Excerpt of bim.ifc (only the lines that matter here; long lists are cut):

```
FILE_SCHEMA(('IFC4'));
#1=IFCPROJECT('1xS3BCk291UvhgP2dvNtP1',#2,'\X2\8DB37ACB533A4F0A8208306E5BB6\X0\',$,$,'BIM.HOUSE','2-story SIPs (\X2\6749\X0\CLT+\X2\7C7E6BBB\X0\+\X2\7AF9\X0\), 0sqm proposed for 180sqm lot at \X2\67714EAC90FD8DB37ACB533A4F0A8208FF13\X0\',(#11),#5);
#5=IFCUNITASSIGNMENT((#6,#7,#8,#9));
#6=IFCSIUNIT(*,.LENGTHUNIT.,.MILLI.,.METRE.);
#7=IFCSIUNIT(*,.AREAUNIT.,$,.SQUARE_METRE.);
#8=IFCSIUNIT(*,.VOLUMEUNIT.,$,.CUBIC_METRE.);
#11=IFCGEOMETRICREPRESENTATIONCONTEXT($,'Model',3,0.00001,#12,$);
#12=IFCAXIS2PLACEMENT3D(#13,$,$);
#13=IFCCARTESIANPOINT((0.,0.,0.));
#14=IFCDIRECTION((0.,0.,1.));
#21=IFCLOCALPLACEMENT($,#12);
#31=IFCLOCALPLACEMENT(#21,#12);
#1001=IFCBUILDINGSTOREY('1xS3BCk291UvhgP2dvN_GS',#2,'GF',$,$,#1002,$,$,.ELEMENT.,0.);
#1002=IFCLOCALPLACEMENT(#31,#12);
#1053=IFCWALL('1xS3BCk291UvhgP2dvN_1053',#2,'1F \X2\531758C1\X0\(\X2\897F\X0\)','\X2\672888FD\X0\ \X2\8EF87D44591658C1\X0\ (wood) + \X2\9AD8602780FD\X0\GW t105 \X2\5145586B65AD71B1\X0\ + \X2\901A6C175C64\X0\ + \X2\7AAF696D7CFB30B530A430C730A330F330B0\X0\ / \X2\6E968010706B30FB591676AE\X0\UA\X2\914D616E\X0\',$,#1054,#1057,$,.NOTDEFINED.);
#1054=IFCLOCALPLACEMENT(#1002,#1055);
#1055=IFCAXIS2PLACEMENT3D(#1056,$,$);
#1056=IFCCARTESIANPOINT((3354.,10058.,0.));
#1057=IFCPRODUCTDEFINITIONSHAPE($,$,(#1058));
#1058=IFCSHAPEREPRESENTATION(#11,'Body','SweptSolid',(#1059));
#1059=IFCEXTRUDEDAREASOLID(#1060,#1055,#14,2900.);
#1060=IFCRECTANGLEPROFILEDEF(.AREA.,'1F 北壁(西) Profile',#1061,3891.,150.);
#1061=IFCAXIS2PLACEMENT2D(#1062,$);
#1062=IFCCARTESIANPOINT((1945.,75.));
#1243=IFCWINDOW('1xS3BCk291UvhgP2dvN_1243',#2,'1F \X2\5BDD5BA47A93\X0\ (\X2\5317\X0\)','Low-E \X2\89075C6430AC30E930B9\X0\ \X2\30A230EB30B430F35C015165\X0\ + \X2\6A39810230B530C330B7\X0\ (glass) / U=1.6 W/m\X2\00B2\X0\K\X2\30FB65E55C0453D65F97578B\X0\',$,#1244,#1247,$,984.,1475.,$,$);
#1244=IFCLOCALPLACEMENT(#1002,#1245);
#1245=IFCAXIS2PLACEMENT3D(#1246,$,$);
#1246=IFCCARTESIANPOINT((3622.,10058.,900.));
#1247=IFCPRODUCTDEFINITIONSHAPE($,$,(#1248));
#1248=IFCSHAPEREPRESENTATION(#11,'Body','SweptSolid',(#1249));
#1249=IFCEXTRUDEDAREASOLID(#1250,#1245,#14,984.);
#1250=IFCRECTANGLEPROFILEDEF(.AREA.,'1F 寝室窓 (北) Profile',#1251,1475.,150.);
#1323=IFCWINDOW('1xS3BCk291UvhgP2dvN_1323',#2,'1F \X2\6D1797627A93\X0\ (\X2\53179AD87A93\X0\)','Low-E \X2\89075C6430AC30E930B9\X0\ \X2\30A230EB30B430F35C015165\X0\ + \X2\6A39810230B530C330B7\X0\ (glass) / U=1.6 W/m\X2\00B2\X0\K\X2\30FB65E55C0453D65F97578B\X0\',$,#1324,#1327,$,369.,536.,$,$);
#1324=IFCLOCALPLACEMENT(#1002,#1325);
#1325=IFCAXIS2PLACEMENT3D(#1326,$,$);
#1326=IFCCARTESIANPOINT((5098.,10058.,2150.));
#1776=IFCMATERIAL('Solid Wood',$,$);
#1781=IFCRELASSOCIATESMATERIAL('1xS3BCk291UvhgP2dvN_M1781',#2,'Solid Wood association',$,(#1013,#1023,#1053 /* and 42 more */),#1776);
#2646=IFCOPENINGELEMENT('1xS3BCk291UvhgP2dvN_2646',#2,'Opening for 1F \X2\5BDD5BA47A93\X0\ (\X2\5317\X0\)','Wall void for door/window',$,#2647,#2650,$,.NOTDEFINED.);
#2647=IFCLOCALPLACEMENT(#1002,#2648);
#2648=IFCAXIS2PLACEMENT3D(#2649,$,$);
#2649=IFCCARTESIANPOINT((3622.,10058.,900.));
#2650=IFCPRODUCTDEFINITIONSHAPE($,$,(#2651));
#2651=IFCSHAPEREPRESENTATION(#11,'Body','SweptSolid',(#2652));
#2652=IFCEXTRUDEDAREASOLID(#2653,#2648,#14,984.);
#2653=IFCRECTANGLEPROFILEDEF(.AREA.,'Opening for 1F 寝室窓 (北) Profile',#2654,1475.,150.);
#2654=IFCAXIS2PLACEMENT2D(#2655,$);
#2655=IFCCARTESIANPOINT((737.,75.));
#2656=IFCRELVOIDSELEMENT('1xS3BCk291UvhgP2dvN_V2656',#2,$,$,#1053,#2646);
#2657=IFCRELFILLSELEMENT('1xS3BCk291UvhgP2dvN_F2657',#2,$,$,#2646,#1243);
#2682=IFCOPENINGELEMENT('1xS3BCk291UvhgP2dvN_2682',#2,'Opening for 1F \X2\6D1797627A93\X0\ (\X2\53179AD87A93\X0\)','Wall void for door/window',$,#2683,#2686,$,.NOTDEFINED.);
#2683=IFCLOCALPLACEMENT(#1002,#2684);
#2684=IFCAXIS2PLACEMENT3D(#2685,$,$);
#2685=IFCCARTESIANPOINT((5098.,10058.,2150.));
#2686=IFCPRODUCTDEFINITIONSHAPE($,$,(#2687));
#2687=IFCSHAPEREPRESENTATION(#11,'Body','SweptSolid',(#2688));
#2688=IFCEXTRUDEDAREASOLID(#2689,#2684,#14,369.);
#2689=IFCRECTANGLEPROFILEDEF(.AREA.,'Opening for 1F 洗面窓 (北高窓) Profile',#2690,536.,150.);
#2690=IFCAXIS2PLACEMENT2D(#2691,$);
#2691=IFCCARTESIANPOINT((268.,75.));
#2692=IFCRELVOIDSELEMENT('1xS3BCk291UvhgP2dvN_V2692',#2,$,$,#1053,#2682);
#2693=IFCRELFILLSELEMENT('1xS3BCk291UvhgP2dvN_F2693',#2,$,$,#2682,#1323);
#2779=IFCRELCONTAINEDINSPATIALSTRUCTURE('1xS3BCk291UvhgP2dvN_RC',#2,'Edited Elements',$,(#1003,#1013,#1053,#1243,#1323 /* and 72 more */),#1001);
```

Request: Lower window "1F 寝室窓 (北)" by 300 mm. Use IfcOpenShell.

```python
import numpy as np
import ifcopenshell
import ifcopenshell.api.geometry
import ifcopenshell.util.placement
import ifcopenshell.util.unit

model = ifcopenshell.open("bim.ifc")
unit_scale = ifcopenshell.util.unit.calculate_unit_scale(model)

window = model.by_guid("1xS3BCk291UvhgP2dvN_1243")
opening = window.FillsVoids[0].RelatingOpeningElement
dz = -0.3 / unit_scale

shift = np.array([0.0, 0.0, dz])
# The window is not placed relative to its opening, so move both.
for product in (opening, window):
    matrix = ifcopenshell.util.placement.get_local_placement(product.ObjectPlacement)
    matrix[:3, 3] += shift
    ifcopenshell.api.geometry.edit_object_placement(model, product=product, matrix=matrix, is_si=False)

print(f"moved by {dz * unit_scale:+.3f} m")

model.write("bim-out.ifc")
```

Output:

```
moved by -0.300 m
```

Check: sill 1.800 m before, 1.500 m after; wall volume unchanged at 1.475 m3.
